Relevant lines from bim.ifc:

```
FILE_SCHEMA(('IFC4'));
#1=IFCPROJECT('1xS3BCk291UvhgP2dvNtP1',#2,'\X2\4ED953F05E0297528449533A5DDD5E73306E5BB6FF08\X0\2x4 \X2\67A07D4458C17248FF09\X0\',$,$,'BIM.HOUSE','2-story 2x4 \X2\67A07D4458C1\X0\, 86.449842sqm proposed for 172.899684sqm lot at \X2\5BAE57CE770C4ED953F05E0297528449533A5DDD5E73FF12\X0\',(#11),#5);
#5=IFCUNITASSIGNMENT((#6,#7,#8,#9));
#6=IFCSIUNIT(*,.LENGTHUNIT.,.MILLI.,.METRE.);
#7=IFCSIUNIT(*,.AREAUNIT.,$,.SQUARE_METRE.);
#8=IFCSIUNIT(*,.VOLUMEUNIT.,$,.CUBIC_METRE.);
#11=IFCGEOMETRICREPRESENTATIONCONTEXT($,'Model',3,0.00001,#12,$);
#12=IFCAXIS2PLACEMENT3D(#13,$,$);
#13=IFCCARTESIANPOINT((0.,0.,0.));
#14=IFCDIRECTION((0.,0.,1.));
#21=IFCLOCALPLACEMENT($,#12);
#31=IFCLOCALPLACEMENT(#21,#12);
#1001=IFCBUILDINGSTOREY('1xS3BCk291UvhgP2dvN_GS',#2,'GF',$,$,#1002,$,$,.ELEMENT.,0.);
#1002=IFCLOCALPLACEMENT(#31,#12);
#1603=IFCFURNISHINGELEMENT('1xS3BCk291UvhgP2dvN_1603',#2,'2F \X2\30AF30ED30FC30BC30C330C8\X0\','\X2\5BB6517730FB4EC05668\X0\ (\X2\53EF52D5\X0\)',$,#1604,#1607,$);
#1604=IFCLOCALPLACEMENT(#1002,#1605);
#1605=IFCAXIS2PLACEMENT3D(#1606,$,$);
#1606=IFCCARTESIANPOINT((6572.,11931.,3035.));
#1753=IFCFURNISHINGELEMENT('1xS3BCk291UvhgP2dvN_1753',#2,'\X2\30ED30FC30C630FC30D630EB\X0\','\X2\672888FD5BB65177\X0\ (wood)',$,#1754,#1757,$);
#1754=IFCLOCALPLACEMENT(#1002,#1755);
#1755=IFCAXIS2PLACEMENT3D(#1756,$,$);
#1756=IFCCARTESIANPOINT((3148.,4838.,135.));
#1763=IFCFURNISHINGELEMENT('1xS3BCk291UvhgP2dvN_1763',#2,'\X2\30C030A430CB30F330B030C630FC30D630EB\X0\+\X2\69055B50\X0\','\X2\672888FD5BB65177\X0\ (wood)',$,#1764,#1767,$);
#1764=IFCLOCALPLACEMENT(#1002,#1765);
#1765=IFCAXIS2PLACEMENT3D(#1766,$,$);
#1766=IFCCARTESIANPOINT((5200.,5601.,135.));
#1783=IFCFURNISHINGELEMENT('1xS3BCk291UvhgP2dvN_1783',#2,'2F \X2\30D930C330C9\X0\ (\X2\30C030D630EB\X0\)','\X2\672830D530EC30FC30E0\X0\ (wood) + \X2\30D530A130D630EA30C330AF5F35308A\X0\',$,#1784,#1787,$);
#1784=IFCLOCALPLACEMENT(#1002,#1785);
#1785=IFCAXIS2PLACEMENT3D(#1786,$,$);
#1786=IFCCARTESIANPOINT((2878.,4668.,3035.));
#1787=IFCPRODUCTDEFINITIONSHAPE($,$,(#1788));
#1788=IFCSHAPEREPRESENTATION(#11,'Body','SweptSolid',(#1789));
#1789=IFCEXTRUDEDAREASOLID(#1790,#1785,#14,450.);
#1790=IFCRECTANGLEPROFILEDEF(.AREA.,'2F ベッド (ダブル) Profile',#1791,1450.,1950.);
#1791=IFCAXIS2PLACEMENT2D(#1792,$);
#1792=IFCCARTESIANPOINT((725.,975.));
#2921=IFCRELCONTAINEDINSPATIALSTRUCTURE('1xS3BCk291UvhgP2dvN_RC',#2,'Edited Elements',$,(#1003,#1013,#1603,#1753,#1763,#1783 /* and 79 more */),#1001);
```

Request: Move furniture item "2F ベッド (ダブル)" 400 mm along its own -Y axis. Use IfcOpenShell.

```python
import ifcopenshell
import ifcopenshell.api.geometry
import ifcopenshell.util.placement
import ifcopenshell.util.unit

model = ifcopenshell.open("bim.ifc")
unit_scale = ifcopenshell.util.unit.calculate_unit_scale(model)

item = model.by_guid("1xS3BCk291UvhgP2dvN_1783")
matrix = ifcopenshell.util.placement.get_local_placement(item.ObjectPlacement)
matrix[:3, 3] -= matrix[:3, 1] * 0.4 / unit_scale
ifcopenshell.api.geometry.edit_object_placement(model, product=item, matrix=matrix, is_si=False)

print(ifcopenshell.util.placement.get_local_placement(item.ObjectPlacement).round(3) + 0.0)

model.write("bim_edited.ifc")
```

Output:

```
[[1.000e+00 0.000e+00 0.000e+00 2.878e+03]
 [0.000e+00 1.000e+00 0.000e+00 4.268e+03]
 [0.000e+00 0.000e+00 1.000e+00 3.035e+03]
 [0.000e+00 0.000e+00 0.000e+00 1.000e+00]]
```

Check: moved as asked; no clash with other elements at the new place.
